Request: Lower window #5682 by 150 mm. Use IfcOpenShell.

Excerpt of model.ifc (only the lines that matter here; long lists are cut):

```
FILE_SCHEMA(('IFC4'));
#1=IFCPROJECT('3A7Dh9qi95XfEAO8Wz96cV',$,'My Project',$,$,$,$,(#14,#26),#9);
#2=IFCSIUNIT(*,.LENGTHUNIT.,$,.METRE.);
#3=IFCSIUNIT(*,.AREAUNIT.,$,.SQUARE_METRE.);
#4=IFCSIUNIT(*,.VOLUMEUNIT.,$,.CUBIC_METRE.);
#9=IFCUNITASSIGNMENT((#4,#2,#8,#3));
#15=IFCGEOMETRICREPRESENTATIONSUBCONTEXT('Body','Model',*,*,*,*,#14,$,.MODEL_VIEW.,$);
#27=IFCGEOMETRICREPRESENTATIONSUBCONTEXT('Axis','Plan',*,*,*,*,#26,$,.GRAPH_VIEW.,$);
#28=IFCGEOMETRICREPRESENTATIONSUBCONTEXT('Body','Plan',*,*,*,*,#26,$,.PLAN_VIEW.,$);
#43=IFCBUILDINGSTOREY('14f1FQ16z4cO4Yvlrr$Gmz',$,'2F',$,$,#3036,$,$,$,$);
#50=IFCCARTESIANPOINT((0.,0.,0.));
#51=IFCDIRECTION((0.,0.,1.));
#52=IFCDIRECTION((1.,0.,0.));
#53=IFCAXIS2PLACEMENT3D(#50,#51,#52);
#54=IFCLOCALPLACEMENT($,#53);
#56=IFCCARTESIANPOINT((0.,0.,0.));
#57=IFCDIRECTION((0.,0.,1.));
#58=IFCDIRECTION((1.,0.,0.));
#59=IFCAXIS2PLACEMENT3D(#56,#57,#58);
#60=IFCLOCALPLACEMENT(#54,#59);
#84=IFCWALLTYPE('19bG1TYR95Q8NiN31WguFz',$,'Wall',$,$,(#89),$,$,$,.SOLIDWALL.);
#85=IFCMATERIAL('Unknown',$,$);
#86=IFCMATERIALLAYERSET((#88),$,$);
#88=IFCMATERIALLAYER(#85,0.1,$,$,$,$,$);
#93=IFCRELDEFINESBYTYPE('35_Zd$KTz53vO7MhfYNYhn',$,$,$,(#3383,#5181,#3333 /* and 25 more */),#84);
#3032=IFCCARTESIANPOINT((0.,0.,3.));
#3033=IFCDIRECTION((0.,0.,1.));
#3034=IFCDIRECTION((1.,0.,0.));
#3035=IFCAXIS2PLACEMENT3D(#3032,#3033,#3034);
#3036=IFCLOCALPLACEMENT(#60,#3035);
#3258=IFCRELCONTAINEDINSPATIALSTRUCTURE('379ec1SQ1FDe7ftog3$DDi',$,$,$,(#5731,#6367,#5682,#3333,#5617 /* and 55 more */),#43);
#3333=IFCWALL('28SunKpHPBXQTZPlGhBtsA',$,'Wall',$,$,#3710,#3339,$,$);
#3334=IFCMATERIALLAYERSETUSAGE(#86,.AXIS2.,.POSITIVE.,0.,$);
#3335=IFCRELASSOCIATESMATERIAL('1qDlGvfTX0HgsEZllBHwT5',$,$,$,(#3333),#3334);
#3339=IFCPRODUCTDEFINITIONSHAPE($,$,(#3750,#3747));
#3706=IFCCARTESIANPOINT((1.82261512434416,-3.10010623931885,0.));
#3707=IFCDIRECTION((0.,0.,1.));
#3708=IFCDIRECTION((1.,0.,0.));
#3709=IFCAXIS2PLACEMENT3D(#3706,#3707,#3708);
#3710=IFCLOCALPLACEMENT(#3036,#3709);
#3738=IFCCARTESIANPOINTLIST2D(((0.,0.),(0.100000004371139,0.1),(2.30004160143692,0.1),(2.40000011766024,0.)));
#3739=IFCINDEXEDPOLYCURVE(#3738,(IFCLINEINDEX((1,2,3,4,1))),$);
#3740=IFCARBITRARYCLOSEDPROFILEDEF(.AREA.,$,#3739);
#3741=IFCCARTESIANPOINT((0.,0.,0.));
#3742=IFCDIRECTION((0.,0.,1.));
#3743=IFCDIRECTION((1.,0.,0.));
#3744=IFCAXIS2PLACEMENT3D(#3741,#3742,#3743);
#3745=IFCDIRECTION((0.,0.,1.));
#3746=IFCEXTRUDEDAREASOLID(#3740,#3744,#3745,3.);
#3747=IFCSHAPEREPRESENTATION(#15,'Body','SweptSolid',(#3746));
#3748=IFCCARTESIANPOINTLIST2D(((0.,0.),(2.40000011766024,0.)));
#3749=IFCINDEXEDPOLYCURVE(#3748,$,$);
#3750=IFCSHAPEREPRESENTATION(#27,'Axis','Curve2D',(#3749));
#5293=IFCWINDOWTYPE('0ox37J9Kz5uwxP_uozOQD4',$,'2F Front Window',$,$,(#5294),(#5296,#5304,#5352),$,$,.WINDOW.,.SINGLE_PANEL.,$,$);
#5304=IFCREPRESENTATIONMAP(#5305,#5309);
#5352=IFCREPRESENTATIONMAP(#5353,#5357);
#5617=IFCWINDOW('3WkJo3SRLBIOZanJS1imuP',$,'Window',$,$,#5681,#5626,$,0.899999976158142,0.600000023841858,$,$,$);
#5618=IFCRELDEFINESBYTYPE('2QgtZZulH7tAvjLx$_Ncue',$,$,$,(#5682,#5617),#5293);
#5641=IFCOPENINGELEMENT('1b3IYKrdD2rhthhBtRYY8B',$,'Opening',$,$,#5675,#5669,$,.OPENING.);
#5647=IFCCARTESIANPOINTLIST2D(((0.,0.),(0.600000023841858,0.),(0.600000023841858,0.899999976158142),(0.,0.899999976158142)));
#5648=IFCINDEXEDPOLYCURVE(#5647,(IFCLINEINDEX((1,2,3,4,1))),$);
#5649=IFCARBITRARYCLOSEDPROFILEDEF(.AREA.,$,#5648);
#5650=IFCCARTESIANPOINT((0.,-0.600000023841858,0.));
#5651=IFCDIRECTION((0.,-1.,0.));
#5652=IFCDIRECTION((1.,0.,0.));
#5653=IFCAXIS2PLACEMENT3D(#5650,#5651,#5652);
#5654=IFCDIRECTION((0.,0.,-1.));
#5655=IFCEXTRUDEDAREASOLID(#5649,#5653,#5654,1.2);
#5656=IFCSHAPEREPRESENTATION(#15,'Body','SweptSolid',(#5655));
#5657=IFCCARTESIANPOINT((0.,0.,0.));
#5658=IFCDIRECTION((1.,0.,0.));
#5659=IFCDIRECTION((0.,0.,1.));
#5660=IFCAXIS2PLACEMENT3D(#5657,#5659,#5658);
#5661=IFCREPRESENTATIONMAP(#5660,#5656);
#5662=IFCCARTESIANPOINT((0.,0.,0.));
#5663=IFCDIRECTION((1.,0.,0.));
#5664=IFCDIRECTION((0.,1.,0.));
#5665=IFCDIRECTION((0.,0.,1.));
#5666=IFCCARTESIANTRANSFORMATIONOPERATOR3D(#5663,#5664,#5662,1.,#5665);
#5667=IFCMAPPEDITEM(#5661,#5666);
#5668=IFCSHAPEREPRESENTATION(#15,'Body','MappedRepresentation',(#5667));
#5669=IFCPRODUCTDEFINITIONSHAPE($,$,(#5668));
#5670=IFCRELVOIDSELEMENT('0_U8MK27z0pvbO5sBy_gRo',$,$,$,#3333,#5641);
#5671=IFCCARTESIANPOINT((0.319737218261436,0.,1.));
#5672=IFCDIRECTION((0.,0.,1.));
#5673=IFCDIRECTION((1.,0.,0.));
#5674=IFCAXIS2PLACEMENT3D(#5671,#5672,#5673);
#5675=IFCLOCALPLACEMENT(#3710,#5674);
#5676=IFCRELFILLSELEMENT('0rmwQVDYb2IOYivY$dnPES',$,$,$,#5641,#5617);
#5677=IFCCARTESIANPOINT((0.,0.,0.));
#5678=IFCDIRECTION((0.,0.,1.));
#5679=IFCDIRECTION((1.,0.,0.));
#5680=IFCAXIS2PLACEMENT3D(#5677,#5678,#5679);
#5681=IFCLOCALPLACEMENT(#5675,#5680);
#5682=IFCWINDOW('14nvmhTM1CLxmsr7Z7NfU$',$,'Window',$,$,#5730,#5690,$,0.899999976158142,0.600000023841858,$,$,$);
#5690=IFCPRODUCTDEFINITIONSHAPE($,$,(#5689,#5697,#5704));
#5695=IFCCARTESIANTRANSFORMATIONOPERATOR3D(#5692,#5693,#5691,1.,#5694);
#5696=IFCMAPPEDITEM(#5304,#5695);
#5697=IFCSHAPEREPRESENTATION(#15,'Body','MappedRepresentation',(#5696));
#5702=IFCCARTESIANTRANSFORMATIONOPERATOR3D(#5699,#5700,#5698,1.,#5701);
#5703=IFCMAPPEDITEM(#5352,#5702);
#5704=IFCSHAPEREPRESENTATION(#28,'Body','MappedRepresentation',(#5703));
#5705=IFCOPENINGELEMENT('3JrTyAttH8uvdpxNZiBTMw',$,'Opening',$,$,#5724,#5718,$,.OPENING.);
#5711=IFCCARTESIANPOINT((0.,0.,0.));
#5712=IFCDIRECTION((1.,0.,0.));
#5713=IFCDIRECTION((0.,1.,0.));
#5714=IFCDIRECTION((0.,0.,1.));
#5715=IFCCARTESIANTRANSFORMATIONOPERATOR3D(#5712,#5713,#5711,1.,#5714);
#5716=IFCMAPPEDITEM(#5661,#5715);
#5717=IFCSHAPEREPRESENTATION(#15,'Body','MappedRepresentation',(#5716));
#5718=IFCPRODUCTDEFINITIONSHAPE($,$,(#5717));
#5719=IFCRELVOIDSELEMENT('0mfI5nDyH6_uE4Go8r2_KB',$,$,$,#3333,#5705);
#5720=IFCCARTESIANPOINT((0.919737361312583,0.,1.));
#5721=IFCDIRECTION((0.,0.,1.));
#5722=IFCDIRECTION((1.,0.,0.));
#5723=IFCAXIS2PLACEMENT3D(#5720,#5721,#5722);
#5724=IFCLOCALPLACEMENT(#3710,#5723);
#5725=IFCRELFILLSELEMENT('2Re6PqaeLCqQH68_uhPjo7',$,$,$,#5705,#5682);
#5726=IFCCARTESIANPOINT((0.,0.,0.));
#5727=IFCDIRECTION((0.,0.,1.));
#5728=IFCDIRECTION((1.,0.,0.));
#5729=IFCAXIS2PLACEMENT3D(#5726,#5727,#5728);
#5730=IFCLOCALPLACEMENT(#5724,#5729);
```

```python
import numpy as np
import ifcopenshell
import ifcopenshell.api.geometry
import ifcopenshell.util.placement
import ifcopenshell.util.unit

model = ifcopenshell.open("model.ifc")
unit_scale = ifcopenshell.util.unit.calculate_unit_scale(model)

window = model.by_id(5682)
opening = window.FillsVoids[0].RelatingOpeningElement
dz = -0.15 / unit_scale

shift = np.array([0.0, 0.0, dz])
# The window is placed relative to its opening, so it follows when the opening moves.
matrix = ifcopenshell.util.placement.get_local_placement(opening.ObjectPlacement)
matrix[:3, 3] += shift
ifcopenshell.api.geometry.edit_object_placement(
    model, product=opening, matrix=matrix, is_si=False, should_transform_children=True
)

print(f"moved by {dz * unit_scale:+.3f} m")

model.write("model_rev.ifc")
```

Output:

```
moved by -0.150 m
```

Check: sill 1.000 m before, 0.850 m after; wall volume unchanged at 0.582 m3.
